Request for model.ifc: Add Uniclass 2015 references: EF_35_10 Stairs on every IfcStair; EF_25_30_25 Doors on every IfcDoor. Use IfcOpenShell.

First a look at what the model holds.

```python
import ifcopenshell

model = ifcopenshell.open("model.ifc")
print(model.schema)
print("classifications:", [c.Name for c in model.by_type("IfcClassification")])
for ifc_class in ("IfcDoor", "IfcRoof", "IfcStair", "IfcWall", "IfcWindow"):
    print(ifc_class, len(model.by_type(ifc_class)))
```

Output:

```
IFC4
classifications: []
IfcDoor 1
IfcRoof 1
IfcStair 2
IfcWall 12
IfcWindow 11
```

```python
import ifcopenshell
import ifcopenshell.api.classification

model = ifcopenshell.open("model.ifc")

system = ifcopenshell.api.classification.add_classification(model, classification="Uniclass 2015")

codes = {
    "IfcStair": ("EF_35_10", "Stairs"),
    "IfcDoor": ("EF_25_30_25", "Doors"),
}
for ifc_class, (code, name) in codes.items():
    products = model.by_type(ifc_class)
    ifcopenshell.api.classification.add_reference(
        model, products=products, classification=system, identification=code, name=name
    )
    print(code, len(products))

model.write("model_updated.ifc")
```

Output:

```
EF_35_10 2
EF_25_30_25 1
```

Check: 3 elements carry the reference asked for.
